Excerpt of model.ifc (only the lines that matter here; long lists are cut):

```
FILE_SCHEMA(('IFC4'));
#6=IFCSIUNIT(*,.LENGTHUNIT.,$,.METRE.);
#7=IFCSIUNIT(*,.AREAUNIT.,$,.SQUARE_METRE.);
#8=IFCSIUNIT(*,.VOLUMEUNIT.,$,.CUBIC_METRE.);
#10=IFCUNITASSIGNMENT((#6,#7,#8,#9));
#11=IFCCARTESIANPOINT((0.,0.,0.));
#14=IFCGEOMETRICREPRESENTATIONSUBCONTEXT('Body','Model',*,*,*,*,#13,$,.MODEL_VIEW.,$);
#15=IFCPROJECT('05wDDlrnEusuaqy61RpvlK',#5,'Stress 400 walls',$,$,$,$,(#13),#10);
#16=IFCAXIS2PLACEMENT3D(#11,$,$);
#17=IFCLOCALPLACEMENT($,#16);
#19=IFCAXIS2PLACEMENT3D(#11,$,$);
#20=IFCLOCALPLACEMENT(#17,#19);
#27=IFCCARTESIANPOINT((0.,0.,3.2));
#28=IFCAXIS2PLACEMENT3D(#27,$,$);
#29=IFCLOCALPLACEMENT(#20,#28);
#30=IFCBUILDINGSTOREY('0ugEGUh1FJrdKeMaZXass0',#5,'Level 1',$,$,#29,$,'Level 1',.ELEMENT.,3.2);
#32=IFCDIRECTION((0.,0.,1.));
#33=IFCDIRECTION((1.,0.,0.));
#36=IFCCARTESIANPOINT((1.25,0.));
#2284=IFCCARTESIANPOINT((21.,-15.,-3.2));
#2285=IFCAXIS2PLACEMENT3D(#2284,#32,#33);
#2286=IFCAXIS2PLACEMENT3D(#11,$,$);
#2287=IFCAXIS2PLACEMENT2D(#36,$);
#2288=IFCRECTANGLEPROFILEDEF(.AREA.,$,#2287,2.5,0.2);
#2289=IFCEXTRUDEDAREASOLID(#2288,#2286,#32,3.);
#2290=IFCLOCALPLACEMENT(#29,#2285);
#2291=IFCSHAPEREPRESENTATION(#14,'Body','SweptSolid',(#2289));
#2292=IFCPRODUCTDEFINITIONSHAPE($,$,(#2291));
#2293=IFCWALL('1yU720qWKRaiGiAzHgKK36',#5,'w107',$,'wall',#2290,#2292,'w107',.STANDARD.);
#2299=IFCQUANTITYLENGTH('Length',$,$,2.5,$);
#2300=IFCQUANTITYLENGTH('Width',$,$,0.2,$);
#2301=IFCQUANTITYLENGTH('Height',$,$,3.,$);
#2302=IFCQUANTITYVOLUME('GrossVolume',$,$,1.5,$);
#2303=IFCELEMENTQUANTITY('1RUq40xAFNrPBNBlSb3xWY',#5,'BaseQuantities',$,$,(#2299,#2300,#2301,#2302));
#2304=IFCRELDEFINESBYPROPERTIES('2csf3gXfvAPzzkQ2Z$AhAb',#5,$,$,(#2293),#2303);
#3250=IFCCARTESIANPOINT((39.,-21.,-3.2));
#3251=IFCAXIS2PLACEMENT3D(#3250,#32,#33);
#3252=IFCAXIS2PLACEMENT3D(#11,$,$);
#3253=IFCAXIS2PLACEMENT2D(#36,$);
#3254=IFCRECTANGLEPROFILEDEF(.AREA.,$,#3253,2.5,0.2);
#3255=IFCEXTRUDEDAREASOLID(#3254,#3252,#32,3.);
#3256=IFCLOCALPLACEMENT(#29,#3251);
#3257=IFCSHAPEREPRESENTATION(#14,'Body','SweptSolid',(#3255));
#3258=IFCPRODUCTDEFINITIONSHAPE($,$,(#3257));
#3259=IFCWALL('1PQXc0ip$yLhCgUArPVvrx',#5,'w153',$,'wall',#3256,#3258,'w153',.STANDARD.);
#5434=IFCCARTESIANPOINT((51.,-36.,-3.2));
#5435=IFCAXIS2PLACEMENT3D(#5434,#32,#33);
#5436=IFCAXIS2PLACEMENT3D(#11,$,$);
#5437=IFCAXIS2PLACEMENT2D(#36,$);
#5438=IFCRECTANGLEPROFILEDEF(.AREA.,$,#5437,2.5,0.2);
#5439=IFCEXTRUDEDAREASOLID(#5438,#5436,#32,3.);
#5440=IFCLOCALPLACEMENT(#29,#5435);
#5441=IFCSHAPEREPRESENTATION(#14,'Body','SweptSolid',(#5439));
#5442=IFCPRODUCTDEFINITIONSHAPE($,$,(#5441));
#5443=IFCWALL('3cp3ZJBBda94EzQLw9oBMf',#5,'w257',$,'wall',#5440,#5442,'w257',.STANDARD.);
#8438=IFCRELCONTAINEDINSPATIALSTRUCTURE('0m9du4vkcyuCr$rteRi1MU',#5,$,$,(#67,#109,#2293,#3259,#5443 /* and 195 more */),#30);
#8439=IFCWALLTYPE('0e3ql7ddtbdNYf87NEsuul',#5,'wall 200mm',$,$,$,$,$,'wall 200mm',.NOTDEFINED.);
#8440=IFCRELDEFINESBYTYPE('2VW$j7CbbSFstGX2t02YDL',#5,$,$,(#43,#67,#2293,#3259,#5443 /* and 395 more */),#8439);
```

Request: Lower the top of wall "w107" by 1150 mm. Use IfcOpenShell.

```python
import ifcopenshell
import ifcopenshell.api.pset
import ifcopenshell.geom
import ifcopenshell.util.element
import ifcopenshell.util.representation
import ifcopenshell.util.shape
import ifcopenshell.util.unit

model = ifcopenshell.open("model.ifc")
unit_scale = ifcopenshell.util.unit.calculate_unit_scale(model)
volume_scale = ifcopenshell.util.unit.calculate_unit_scale(model, "VOLUMEUNIT")
settings = ifcopenshell.geom.settings()


def volume(element):
    """Net volume in cubic metres, openings subtracted."""
    shape = ifcopenshell.geom.create_shape(settings, element)
    return ifcopenshell.util.shape.get_volume(shape.geometry)


wall = model.by_guid("1yU720qWKRaiGiAzHgKK36")
before = volume(wall)

body = ifcopenshell.util.representation.get_representation(wall, "Model", "Body")
solid = body.Items[0]
old_height = solid.Depth
solid.Depth -= 1.15
after = volume(wall)

# Update the stored height, areas and volumes.
qto = model.by_id(ifcopenshell.util.element.get_pset(wall, "BaseQuantities", should_inherit=False)["id"])
ifcopenshell.api.pset.edit_qto(model, qto=qto, properties={
    "Height": solid.Depth,
    "GrossVolume": ifcopenshell.util.element.get_pset(wall, "BaseQuantities", "GrossVolume") * solid.Depth / old_height,
})

print(f"height {old_height:g} -> {solid.Depth:g}, volume {before:.3f} -> {after:.3f} m3")

model.write("model-out.ifc")
```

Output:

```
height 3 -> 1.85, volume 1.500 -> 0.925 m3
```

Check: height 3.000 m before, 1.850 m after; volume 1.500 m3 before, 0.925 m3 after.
